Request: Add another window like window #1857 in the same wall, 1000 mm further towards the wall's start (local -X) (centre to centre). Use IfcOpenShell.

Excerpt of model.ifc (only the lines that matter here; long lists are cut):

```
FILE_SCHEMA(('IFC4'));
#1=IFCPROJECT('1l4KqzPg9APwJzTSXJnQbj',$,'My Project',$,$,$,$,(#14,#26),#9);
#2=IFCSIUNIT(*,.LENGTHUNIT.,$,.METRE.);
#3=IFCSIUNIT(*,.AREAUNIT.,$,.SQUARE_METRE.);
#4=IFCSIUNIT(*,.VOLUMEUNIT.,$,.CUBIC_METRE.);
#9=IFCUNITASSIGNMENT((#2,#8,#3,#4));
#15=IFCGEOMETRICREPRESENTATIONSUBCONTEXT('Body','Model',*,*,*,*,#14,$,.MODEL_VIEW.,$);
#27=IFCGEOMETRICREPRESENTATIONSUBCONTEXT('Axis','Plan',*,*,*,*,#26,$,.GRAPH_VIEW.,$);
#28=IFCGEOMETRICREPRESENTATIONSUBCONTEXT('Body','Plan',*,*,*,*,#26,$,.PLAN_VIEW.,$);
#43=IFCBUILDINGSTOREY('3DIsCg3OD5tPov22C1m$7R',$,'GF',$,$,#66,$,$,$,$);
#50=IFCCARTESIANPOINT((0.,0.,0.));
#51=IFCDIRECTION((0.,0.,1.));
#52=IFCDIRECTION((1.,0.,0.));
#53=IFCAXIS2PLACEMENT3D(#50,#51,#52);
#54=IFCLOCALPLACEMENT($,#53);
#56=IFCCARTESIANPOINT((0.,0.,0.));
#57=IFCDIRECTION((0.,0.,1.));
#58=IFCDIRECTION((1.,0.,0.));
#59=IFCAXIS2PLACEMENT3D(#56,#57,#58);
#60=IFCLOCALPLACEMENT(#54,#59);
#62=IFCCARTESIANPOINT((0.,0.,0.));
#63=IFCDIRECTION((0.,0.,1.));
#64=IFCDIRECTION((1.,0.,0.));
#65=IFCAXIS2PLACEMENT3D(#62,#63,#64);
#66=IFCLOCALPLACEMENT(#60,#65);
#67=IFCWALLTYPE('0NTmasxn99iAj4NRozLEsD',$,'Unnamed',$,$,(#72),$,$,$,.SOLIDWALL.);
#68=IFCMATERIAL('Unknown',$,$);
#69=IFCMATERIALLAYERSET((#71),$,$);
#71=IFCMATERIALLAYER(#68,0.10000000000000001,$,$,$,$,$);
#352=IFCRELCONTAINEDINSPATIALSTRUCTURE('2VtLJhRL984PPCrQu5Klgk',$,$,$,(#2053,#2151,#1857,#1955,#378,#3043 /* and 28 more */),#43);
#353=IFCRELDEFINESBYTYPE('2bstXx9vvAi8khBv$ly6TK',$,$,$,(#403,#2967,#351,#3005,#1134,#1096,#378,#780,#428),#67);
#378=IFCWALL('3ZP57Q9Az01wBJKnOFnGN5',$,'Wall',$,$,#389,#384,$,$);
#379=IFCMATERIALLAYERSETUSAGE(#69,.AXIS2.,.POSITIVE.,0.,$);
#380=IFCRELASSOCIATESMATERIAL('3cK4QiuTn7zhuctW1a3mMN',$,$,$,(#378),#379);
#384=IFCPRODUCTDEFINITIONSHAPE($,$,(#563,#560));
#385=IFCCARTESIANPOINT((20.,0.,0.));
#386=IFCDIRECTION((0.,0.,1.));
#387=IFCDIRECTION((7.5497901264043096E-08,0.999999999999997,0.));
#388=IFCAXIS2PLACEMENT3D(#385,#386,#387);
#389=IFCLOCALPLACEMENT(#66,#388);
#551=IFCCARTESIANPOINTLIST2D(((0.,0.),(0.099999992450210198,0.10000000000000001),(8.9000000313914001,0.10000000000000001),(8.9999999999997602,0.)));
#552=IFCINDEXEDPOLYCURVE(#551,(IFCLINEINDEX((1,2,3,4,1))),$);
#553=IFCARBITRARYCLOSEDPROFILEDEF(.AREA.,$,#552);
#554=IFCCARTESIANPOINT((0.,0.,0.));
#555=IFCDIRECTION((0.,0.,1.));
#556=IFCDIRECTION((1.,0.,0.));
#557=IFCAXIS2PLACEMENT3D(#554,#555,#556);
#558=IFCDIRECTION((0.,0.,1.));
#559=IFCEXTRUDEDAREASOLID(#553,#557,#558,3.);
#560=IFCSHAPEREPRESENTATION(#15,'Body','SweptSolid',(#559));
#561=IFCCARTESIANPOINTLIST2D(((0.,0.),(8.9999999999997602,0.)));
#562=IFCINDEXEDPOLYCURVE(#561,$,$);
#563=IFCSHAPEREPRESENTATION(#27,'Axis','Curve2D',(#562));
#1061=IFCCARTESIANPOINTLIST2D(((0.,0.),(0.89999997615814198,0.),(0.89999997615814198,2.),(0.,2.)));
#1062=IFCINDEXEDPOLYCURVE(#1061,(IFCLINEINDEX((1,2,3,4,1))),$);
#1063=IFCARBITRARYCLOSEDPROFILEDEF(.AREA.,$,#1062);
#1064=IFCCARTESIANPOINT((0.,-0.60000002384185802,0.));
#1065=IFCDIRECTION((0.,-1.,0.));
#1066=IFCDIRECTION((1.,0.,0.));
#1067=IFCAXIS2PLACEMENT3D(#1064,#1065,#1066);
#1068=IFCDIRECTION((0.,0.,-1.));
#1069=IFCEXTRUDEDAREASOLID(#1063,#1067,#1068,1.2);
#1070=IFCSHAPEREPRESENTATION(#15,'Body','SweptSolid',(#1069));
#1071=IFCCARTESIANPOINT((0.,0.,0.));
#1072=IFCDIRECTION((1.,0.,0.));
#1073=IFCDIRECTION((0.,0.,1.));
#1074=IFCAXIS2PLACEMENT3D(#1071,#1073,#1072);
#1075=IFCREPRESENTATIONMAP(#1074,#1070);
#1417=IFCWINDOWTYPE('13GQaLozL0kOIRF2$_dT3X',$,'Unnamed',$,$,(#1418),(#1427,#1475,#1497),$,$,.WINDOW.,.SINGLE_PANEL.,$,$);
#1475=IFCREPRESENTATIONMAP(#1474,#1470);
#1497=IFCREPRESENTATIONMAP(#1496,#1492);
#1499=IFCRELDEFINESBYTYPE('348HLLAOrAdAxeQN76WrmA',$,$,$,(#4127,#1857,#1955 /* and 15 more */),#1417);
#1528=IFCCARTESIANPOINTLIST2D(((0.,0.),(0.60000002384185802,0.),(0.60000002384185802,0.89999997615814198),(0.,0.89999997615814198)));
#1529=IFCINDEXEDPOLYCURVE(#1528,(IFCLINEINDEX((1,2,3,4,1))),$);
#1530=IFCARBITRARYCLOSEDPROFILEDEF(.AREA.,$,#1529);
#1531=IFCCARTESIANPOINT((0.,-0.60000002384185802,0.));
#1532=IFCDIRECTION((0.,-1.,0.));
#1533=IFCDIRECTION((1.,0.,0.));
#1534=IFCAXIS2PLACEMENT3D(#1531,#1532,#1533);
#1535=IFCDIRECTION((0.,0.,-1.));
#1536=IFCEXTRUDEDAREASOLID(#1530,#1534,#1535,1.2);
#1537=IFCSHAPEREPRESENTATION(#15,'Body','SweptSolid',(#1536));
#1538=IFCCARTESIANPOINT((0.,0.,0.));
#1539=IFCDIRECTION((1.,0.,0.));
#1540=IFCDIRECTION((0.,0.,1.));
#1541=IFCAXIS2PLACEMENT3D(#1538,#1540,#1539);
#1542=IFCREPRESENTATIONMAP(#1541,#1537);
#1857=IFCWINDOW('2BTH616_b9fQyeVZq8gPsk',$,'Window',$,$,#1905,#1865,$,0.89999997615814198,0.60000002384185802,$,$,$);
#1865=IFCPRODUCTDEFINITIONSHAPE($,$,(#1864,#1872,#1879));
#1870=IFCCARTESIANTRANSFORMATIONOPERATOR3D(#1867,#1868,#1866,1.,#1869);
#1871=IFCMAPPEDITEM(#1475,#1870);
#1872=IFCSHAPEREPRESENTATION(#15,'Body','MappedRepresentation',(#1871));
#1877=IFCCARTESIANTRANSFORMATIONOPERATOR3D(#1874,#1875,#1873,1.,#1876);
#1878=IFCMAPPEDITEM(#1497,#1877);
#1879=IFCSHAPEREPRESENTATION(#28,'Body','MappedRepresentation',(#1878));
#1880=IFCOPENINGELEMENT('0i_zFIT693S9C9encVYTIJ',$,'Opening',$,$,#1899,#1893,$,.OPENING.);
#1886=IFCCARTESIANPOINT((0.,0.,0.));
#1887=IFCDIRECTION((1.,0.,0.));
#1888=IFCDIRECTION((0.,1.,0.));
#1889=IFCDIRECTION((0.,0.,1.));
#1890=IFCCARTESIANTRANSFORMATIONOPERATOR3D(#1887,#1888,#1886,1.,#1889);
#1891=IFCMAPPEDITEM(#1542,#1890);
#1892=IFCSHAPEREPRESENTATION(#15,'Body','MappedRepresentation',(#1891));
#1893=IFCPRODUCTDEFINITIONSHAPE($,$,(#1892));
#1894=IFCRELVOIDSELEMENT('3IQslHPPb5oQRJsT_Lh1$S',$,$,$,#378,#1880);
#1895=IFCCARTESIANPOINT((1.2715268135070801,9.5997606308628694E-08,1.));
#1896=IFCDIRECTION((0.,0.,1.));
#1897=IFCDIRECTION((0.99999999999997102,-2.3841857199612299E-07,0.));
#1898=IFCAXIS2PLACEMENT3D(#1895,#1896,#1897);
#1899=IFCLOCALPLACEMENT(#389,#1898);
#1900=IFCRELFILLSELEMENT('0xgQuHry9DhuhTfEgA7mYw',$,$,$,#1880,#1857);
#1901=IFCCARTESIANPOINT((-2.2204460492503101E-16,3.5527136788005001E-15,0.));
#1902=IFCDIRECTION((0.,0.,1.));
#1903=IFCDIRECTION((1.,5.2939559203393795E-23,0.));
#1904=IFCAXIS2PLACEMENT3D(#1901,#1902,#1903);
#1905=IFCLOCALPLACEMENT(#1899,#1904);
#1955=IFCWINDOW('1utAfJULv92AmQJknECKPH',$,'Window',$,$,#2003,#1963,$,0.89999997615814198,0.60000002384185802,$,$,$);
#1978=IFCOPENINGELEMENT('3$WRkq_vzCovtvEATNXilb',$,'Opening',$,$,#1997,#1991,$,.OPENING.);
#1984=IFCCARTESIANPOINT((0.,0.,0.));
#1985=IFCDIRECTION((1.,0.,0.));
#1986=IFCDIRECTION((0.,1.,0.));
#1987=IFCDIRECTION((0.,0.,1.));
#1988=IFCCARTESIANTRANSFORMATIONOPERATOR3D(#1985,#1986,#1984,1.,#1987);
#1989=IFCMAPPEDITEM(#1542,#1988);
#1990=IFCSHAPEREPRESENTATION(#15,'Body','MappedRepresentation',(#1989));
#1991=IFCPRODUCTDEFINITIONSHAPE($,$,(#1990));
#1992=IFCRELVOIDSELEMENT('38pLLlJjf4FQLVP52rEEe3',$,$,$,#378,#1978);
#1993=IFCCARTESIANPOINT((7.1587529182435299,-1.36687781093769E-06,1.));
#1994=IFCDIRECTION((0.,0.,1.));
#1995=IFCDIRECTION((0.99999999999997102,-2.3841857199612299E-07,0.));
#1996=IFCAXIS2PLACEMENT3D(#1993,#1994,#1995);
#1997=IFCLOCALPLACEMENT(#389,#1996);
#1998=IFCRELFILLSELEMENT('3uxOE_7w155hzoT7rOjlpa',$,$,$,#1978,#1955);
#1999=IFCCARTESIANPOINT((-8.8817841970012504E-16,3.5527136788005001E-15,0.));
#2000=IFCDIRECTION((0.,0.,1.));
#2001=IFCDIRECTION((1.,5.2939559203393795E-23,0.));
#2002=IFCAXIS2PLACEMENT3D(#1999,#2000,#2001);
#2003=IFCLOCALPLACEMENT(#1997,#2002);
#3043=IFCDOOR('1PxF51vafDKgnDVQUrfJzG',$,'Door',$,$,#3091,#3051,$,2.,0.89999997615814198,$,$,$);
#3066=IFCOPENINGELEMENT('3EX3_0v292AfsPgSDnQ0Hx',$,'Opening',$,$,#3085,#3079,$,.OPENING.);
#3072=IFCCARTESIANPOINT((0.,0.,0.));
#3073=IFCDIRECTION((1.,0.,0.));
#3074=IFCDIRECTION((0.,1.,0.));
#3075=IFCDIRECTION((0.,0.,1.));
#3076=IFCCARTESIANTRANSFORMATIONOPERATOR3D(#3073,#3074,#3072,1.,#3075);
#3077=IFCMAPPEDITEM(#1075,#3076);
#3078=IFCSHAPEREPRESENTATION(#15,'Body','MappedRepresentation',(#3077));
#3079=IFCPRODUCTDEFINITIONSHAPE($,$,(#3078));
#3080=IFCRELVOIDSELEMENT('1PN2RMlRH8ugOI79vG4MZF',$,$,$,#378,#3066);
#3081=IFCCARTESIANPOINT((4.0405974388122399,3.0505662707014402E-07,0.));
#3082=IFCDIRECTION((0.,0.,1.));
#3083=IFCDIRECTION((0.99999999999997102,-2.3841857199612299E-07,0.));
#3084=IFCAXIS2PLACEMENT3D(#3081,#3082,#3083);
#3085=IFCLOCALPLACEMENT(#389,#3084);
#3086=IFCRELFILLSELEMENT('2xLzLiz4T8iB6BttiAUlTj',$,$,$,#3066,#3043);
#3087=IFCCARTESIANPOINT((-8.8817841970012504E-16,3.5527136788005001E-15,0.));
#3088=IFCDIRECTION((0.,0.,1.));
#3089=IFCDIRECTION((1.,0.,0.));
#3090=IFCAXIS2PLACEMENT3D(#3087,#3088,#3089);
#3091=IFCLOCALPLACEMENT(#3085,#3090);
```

```python
import ifcopenshell
import ifcopenshell.api.feature
import ifcopenshell.api.geometry
import ifcopenshell.api.root
import ifcopenshell.geom
import ifcopenshell.util.element
import ifcopenshell.util.placement
import ifcopenshell.util.shape

model = ifcopenshell.open("model.ifc")
settings = ifcopenshell.geom.settings()


def volume(element):
    """Net volume in cubic metres, openings subtracted."""
    shape = ifcopenshell.geom.create_shape(settings, element)
    return ifcopenshell.util.shape.get_volume(shape.geometry)


window = model.by_guid("2BTH616_b9fQyeVZq8gPsk")
opening = window.FillsVoids[0].RelatingOpeningElement
wall = opening.VoidsElements[0].RelatingBuildingElement
before = volume(wall)
shift = ifcopenshell.util.placement.get_local_placement(wall.ObjectPlacement)[:3, 0] * -1.0

# copy_class copies the void relationship, type, container and properties, but no geometry.
new_opening = ifcopenshell.api.root.copy_class(model, product=opening)
new_opening.Representation = ifcopenshell.util.element.copy_deep(
    model, opening.Representation, exclude=["IfcGeometricRepresentationContext", "IfcRepresentationMap"]
)
new_window = ifcopenshell.api.root.copy_class(model, product=window)
new_window.Representation = ifcopenshell.util.element.copy_deep(
    model, window.Representation, exclude=["IfcGeometricRepresentationContext", "IfcRepresentationMap"]
)
ifcopenshell.api.feature.add_filling(model, opening=new_opening, element=new_window)

for old, new in ((opening, new_opening), (window, new_window)):
    matrix = ifcopenshell.util.placement.get_local_placement(old.ObjectPlacement)
    matrix[:3, 3] += shift
    ifcopenshell.api.geometry.edit_object_placement(model, product=new, matrix=matrix, is_si=False)

after = volume(wall)

print(f"wall volume {before:.3f} -> {after:.3f} m3")

model.write("model_v2.ifc")
```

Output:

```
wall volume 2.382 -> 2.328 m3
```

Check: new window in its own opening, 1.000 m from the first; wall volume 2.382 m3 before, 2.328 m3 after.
